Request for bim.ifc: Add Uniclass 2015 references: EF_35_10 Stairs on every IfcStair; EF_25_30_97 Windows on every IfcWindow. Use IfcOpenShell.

First a look at what the model holds.

```python
import ifcopenshell

model = ifcopenshell.open("bim.ifc")
print(model.schema)
print("classifications:", [c.Name for c in model.by_type("IfcClassification")])
for ifc_class in ("IfcDoor", "IfcRoof", "IfcStair", "IfcWall", "IfcWindow"):
    print(ifc_class, len(model.by_type(ifc_class)))
```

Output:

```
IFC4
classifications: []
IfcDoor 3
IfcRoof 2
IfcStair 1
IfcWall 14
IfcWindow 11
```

```python
import ifcopenshell
import ifcopenshell.api.classification

model = ifcopenshell.open("bim.ifc")

system = ifcopenshell.api.classification.add_classification(model, classification="Uniclass 2015")

codes = {
    "IfcStair": ("EF_35_10", "Stairs"),
    "IfcWindow": ("EF_25_30_97", "Windows"),
}
for ifc_class, (code, name) in codes.items():
    products = model.by_type(ifc_class)
    ifcopenshell.api.classification.add_reference(
        model, products=products, classification=system, identification=code, name=name
    )
    print(code, len(products))

model.write("bim_rev.ifc")
```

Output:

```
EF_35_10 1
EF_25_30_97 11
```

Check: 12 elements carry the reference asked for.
